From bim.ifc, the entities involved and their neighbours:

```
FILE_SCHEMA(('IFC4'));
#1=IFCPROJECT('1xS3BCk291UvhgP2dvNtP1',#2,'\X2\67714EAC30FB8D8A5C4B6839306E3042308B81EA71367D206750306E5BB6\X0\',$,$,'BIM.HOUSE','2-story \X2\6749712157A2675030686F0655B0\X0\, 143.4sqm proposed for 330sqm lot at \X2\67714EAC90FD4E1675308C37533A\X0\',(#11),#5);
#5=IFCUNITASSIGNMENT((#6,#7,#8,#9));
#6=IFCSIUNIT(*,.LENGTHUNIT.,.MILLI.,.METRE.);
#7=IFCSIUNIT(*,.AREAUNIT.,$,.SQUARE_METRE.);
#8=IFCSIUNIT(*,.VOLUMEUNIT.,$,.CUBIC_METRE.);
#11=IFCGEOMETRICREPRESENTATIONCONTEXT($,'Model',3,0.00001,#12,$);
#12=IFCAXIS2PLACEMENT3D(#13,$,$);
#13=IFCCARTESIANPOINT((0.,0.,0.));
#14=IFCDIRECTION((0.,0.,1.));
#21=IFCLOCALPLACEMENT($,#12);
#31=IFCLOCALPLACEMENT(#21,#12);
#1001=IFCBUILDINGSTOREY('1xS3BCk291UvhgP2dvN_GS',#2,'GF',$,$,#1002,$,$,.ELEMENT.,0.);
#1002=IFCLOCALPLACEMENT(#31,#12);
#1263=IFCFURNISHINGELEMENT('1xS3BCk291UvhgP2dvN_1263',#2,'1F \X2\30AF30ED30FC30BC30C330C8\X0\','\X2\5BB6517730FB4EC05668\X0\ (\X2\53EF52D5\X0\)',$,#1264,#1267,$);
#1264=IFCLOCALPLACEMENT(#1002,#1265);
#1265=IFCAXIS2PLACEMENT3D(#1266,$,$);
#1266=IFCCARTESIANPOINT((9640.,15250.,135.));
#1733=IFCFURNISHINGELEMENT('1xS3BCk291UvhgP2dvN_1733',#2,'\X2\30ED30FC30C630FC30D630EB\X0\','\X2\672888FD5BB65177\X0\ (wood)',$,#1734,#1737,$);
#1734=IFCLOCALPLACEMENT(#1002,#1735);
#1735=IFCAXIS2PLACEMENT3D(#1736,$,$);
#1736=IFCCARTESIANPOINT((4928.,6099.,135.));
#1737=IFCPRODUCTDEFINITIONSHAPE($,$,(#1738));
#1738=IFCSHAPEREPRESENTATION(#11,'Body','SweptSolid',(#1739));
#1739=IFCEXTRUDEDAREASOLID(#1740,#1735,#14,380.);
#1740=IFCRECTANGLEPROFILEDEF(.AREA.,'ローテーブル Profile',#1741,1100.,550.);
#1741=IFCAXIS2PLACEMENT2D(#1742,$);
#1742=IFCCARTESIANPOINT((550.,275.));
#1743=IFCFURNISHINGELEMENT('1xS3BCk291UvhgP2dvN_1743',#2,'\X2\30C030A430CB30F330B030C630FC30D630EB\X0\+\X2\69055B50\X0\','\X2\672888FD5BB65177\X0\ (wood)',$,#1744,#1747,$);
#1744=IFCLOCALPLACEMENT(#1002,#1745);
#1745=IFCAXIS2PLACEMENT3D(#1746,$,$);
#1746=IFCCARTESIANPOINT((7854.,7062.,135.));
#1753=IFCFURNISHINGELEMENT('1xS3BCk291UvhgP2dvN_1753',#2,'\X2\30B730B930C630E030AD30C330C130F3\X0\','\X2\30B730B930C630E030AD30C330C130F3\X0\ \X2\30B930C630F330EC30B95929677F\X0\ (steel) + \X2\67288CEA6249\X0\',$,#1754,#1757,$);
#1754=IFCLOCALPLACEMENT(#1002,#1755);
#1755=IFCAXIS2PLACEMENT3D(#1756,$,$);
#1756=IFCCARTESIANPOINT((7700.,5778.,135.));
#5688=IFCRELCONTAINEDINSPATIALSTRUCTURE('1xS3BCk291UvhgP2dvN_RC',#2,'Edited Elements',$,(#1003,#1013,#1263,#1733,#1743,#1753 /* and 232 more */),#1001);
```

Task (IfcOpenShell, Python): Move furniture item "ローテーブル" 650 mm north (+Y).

```python
import ifcopenshell
import ifcopenshell.api.geometry
import ifcopenshell.util.placement
import ifcopenshell.util.unit

model = ifcopenshell.open("bim.ifc")
unit_scale = ifcopenshell.util.unit.calculate_unit_scale(model)

item = model.by_guid("1xS3BCk291UvhgP2dvN_1733")
matrix = ifcopenshell.util.placement.get_local_placement(item.ObjectPlacement)
matrix[1, 3] += 0.65 / unit_scale
ifcopenshell.api.geometry.edit_object_placement(model, product=item, matrix=matrix, is_si=False)

print(ifcopenshell.util.placement.get_local_placement(item.ObjectPlacement).round(3) + 0.0)

model.write("bim_v2.ifc")
```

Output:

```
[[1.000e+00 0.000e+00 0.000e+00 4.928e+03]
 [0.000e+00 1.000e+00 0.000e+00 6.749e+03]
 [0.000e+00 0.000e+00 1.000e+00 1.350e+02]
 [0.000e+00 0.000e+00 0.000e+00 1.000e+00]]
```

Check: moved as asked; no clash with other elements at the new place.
